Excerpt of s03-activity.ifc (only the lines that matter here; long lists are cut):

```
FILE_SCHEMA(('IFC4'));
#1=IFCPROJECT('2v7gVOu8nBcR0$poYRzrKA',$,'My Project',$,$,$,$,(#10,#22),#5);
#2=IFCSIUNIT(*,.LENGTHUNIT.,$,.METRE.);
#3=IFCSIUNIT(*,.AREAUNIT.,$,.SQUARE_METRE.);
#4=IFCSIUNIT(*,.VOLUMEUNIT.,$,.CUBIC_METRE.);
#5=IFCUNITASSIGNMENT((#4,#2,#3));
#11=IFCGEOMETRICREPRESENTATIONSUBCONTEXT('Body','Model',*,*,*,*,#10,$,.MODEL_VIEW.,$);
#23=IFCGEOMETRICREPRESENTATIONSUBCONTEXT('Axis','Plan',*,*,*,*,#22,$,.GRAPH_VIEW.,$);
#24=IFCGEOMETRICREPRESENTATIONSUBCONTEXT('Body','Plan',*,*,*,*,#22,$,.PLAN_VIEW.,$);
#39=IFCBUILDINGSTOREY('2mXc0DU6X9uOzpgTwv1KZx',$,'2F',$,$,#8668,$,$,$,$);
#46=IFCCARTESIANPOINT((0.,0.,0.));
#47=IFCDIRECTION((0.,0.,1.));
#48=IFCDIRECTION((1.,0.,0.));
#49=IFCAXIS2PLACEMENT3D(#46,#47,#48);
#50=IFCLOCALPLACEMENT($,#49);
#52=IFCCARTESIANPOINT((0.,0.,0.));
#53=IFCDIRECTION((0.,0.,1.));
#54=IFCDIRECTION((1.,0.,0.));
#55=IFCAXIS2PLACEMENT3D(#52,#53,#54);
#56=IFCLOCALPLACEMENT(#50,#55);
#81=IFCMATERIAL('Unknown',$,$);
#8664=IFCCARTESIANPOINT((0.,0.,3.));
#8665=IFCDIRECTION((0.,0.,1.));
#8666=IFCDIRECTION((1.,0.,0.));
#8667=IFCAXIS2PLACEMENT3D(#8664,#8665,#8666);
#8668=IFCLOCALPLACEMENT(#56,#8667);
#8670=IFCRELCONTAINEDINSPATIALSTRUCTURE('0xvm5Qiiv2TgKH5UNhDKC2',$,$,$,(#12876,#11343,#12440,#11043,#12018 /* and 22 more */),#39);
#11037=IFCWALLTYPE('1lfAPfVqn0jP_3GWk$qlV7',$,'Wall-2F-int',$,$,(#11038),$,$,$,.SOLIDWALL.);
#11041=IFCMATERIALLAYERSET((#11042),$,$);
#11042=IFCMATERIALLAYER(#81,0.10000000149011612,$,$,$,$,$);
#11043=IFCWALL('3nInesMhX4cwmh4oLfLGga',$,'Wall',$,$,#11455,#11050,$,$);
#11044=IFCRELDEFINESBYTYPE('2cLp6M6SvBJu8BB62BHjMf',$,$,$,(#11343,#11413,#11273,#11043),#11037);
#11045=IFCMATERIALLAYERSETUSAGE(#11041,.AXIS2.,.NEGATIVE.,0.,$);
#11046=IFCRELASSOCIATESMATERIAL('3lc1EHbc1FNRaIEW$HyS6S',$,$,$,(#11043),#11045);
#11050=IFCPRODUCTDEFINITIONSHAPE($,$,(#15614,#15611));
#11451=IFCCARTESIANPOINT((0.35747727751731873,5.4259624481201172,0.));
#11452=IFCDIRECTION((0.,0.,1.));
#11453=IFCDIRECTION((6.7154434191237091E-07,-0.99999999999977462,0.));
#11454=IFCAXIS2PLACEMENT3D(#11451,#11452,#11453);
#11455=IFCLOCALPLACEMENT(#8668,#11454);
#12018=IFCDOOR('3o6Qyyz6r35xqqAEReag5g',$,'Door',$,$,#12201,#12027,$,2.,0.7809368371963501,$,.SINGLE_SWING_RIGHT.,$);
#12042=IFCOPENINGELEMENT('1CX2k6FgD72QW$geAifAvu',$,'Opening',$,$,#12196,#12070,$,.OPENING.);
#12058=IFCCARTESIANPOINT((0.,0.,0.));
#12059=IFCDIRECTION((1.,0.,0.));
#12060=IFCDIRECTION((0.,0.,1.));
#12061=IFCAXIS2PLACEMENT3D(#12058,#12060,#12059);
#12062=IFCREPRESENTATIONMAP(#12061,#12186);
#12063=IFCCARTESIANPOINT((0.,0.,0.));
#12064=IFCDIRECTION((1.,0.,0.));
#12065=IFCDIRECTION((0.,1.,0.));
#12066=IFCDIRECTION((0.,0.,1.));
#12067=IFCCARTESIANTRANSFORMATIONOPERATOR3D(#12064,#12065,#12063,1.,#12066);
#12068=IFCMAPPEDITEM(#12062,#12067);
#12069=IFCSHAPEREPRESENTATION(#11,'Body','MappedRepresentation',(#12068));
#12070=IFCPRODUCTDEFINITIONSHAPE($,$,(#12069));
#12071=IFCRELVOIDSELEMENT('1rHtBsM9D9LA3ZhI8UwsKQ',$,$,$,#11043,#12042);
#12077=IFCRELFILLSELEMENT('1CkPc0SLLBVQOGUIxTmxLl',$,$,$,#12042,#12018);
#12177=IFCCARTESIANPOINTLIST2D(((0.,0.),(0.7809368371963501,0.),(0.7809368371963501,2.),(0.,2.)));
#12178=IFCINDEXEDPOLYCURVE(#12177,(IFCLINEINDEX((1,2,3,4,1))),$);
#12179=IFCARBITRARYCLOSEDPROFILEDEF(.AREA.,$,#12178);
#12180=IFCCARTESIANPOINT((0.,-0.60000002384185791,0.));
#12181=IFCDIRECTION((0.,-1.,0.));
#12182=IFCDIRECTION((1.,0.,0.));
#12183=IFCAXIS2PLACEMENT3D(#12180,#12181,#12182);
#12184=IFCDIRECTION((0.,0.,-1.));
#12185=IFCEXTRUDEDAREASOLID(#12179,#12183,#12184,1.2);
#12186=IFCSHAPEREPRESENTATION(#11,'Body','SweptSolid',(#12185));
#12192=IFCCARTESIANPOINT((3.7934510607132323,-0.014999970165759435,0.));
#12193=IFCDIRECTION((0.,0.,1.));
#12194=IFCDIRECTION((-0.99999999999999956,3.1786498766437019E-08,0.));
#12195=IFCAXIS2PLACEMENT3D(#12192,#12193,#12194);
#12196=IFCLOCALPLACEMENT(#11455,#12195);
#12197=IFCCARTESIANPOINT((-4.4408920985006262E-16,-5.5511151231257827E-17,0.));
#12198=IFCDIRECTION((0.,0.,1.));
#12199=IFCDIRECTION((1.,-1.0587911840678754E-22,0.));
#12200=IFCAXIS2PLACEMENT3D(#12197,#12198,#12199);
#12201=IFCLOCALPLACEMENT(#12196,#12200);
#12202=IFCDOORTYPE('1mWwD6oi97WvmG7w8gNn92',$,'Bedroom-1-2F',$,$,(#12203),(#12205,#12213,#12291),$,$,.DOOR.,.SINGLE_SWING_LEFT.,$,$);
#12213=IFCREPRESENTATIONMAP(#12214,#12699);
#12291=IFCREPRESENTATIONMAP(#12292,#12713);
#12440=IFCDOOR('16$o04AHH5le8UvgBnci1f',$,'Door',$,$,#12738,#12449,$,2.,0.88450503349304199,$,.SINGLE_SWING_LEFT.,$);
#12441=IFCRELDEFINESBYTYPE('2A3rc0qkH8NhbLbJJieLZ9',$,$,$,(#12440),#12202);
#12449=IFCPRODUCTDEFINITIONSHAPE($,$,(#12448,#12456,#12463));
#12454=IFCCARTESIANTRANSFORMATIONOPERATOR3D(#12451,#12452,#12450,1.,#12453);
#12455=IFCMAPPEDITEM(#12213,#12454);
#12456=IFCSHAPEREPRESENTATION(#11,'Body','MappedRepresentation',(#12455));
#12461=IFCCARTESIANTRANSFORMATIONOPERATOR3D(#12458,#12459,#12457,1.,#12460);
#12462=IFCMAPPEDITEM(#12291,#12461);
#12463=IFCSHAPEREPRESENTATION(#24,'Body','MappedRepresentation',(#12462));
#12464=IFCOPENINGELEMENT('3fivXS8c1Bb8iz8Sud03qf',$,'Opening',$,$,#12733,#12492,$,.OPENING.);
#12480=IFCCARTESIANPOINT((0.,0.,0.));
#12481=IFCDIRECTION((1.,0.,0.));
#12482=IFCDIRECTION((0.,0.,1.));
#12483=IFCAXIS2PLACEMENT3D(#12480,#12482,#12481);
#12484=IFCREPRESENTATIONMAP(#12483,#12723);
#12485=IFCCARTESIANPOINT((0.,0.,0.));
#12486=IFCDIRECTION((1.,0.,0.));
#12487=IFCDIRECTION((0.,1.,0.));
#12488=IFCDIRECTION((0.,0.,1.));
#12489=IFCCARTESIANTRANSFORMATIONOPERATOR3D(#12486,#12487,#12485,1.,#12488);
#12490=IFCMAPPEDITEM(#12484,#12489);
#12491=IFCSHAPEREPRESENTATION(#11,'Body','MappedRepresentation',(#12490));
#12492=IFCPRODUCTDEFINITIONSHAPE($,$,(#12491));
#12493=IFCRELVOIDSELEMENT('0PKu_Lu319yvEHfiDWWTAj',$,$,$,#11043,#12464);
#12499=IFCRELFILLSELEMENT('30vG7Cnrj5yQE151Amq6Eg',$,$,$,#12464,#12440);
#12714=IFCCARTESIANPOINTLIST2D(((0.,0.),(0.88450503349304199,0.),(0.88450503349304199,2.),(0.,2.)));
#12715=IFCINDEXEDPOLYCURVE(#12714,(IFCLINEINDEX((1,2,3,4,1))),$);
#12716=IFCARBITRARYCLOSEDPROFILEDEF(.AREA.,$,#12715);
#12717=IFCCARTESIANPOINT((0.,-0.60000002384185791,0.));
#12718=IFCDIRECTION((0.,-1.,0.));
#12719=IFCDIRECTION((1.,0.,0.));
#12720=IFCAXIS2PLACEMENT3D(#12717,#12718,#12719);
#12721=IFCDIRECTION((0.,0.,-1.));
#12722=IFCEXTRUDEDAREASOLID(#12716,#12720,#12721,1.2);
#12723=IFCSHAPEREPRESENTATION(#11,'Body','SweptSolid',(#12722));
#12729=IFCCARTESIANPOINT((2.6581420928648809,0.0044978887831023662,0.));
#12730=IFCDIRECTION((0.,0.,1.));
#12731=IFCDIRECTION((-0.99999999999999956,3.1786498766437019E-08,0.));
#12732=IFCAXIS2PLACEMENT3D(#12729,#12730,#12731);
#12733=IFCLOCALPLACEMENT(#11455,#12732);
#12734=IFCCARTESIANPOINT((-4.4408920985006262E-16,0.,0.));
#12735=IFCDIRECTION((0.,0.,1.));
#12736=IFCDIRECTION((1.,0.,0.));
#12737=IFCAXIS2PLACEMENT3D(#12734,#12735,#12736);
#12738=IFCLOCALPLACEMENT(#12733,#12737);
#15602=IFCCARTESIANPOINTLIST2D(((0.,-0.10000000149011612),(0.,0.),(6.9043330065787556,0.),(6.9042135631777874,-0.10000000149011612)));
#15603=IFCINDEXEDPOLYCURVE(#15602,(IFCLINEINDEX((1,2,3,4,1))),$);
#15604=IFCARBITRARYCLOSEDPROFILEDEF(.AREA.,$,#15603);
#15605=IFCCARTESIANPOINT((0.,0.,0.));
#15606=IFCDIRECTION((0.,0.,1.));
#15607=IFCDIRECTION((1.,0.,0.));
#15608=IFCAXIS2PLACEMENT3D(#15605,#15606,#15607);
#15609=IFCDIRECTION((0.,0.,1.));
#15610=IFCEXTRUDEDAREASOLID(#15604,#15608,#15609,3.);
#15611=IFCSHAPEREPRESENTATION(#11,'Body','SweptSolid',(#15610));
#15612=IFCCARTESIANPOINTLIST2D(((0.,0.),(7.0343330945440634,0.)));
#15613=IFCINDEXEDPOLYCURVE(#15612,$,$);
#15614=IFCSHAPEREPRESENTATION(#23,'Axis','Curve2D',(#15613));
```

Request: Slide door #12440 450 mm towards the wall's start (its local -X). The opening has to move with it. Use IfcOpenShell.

```python
import ifcopenshell
import ifcopenshell.api.geometry
import ifcopenshell.util.placement

model = ifcopenshell.open("s03-activity.ifc")

door = model.by_guid("16$o04AHH5le8UvgBnci1f")
opening = door.FillsVoids[0].RelatingOpeningElement
wall = opening.VoidsElements[0].RelatingBuildingElement

wall_matrix = ifcopenshell.util.placement.get_local_placement(wall.ObjectPlacement)
shift = wall_matrix[:3, 0] * -0.45
before = ifcopenshell.util.placement.get_local_placement(door.ObjectPlacement)[:3, 3].copy()

# The door is placed relative to its opening, so it follows when the opening moves.
matrix = ifcopenshell.util.placement.get_local_placement(opening.ObjectPlacement)
matrix[:3, 3] += shift
ifcopenshell.api.geometry.edit_object_placement(
    model, product=opening, matrix=matrix, is_si=False, should_transform_children=True
)

after = ifcopenshell.util.placement.get_local_placement(door.ObjectPlacement)[:3, 3]
print("door moved by", (after - before).round(3) + 0.0)

model.write("s03-activity_edited.ifc")
```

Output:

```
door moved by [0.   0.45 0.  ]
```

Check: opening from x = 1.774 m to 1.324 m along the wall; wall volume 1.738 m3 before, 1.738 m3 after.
